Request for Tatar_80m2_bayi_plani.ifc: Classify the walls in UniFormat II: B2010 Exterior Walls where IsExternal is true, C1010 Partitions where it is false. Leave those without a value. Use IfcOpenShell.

First a look at what the model holds.

```python
import ifcopenshell
import ifcopenshell.util.element

model = ifcopenshell.open("Tatar_80m2_bayi_plani.ifc")
print(model.schema)
print("classifications:", [c.Name for c in model.by_type("IfcClassification")])
values = [ifcopenshell.util.element.get_pset(e, "Pset_WallCommon", "IsExternal") for e in model.by_type("IfcWall")]
for value in (True, False, None):
    print("IsExternal", value, values.count(value))
```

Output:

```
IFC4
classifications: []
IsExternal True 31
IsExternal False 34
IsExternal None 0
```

```python
import ifcopenshell
import ifcopenshell.api.classification
import ifcopenshell.util.element

model = ifcopenshell.open("Tatar_80m2_bayi_plani.ifc")

system = ifcopenshell.api.classification.add_classification(model, classification="UniFormat II")

walls = model.by_type("IfcWall")
external = {e: ifcopenshell.util.element.get_pset(e, "Pset_WallCommon", "IsExternal") for e in walls}
for flag, code, name in ((True, "B2010", "Exterior Walls"), (False, "C1010", "Partitions")):
    products = [e for e in walls if external[e] is flag]
    ifcopenshell.api.classification.add_reference(
        model, products=products, classification=system, identification=code, name=name
    )
    print(code, len(products))

model.write("Tatar_80m2_bayi_plani_rev.ifc")
```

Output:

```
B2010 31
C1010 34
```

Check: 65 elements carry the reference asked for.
